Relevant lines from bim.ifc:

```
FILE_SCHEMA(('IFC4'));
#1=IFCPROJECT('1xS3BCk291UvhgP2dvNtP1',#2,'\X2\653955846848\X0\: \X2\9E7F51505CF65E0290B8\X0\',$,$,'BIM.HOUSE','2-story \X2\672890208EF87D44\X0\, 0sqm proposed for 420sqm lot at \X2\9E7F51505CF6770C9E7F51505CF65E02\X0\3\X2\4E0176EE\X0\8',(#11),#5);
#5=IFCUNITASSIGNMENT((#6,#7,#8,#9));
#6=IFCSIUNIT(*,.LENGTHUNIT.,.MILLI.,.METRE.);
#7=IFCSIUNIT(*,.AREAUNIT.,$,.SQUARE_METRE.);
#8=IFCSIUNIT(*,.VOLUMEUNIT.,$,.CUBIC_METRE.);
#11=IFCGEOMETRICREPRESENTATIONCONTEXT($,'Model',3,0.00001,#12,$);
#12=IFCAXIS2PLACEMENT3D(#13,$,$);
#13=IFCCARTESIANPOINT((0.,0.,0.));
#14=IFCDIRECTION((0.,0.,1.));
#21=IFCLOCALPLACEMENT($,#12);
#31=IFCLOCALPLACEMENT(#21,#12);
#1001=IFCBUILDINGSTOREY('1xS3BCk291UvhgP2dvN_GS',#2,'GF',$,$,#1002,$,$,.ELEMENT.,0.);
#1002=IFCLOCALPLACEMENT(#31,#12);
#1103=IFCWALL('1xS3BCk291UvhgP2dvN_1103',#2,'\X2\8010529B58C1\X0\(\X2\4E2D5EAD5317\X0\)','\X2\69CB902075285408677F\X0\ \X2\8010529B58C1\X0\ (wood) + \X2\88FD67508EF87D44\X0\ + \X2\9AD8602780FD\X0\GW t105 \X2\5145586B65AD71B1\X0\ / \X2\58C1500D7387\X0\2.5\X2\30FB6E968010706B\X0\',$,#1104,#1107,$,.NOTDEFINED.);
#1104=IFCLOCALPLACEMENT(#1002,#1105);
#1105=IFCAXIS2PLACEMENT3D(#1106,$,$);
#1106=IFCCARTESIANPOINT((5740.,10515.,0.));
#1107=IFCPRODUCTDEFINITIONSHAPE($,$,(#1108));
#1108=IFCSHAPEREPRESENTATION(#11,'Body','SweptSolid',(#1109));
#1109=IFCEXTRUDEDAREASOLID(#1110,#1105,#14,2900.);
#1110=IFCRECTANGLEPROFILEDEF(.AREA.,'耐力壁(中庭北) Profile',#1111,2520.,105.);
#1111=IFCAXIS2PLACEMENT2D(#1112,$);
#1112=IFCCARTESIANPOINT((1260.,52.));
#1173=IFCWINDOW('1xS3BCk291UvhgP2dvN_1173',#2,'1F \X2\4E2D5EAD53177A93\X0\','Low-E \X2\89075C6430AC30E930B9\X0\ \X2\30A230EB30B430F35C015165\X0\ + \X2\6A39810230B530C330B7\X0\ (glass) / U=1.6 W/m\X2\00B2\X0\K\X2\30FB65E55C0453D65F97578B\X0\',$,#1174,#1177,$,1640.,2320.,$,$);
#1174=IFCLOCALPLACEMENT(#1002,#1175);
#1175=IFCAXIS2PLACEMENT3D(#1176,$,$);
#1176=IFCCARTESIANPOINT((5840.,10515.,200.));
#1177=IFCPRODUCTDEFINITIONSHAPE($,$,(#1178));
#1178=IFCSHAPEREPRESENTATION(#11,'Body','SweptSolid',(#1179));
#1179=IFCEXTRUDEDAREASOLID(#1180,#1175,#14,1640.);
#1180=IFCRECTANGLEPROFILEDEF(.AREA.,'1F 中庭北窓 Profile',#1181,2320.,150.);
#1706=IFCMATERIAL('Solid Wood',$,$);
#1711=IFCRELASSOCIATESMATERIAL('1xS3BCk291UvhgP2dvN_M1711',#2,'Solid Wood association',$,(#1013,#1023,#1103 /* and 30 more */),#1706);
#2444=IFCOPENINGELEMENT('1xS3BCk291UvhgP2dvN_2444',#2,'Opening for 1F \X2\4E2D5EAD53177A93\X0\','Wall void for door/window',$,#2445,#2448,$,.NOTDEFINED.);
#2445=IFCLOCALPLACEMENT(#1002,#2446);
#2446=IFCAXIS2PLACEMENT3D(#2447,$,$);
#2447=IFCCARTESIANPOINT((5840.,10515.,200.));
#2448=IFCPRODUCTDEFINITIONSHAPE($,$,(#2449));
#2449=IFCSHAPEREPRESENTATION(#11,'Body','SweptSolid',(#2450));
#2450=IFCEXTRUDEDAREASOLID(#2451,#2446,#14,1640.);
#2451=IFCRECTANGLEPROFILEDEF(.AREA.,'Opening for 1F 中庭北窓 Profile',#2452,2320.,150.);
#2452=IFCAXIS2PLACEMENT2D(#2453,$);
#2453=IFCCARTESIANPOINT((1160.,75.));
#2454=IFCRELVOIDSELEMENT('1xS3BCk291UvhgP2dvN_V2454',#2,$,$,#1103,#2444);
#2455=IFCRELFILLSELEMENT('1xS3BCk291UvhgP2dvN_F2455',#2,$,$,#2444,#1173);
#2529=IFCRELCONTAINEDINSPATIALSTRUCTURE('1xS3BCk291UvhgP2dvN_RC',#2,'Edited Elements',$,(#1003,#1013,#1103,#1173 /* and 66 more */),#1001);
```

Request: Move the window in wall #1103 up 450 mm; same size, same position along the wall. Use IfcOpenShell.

```python
import numpy as np
import ifcopenshell
import ifcopenshell.api.geometry
import ifcopenshell.util.placement
import ifcopenshell.util.unit

model = ifcopenshell.open("bim.ifc")
unit_scale = ifcopenshell.util.unit.calculate_unit_scale(model)

window = model.by_guid("1xS3BCk291UvhgP2dvN_1173")
opening = window.FillsVoids[0].RelatingOpeningElement
dz = 0.45 / unit_scale

shift = np.array([0.0, 0.0, dz])
# The window is not placed relative to its opening, so move both.
for product in (opening, window):
    matrix = ifcopenshell.util.placement.get_local_placement(product.ObjectPlacement)
    matrix[:3, 3] += shift
    ifcopenshell.api.geometry.edit_object_placement(model, product=product, matrix=matrix, is_si=False)

print(f"moved by {dz * unit_scale:+.3f} m")

model.write("bim_edited.ifc")
```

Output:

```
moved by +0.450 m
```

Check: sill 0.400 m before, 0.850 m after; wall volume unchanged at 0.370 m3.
